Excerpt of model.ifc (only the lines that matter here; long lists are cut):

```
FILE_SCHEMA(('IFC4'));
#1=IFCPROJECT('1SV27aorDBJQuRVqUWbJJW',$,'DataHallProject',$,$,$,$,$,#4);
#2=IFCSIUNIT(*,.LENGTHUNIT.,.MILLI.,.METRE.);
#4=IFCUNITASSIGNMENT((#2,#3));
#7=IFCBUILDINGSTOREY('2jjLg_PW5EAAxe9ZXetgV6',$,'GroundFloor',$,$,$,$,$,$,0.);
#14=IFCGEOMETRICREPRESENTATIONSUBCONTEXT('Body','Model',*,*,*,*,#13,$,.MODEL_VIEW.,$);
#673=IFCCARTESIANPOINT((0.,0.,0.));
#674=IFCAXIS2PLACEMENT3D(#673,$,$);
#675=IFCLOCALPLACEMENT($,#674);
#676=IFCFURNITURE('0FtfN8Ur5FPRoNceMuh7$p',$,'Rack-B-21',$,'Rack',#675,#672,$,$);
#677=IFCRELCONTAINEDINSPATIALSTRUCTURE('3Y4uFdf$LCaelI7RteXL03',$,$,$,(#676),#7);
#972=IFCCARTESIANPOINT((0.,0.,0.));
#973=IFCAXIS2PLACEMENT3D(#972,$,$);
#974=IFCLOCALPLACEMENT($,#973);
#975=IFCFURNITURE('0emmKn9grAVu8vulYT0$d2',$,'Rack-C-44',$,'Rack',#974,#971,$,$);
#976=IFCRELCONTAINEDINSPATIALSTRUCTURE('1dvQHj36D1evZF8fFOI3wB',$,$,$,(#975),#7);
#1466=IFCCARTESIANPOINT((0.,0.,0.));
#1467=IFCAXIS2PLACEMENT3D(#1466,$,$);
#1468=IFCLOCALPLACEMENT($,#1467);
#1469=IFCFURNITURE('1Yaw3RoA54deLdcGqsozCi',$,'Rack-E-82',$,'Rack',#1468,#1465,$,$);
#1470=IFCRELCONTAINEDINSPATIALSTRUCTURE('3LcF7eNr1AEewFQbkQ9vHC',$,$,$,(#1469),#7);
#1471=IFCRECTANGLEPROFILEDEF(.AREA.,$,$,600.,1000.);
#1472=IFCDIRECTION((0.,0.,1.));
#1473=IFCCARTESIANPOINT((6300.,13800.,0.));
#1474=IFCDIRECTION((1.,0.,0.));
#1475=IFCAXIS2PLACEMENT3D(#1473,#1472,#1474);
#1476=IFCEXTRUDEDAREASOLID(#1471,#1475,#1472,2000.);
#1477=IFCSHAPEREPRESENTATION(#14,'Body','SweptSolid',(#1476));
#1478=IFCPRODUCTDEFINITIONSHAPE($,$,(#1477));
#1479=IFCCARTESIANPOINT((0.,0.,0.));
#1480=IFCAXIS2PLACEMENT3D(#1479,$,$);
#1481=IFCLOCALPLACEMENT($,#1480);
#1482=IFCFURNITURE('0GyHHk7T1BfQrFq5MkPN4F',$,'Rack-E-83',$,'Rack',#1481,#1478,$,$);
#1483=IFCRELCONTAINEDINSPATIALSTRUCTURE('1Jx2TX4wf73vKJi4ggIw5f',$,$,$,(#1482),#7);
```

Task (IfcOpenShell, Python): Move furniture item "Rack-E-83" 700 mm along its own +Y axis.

```python
import ifcopenshell
import ifcopenshell.api.geometry
import ifcopenshell.util.placement
import ifcopenshell.util.unit

model = ifcopenshell.open("model.ifc")
unit_scale = ifcopenshell.util.unit.calculate_unit_scale(model)

item = model.by_id(1482)
matrix = ifcopenshell.util.placement.get_local_placement(item.ObjectPlacement)
matrix[:3, 3] += matrix[:3, 1] * 0.7 / unit_scale
ifcopenshell.api.geometry.edit_object_placement(model, product=item, matrix=matrix, is_si=False)

print(ifcopenshell.util.placement.get_local_placement(item.ObjectPlacement).round(3) + 0.0)

model.write("model_edited.ifc")
```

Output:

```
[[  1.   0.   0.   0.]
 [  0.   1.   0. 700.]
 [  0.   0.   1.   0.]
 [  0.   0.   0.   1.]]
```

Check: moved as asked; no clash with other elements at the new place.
